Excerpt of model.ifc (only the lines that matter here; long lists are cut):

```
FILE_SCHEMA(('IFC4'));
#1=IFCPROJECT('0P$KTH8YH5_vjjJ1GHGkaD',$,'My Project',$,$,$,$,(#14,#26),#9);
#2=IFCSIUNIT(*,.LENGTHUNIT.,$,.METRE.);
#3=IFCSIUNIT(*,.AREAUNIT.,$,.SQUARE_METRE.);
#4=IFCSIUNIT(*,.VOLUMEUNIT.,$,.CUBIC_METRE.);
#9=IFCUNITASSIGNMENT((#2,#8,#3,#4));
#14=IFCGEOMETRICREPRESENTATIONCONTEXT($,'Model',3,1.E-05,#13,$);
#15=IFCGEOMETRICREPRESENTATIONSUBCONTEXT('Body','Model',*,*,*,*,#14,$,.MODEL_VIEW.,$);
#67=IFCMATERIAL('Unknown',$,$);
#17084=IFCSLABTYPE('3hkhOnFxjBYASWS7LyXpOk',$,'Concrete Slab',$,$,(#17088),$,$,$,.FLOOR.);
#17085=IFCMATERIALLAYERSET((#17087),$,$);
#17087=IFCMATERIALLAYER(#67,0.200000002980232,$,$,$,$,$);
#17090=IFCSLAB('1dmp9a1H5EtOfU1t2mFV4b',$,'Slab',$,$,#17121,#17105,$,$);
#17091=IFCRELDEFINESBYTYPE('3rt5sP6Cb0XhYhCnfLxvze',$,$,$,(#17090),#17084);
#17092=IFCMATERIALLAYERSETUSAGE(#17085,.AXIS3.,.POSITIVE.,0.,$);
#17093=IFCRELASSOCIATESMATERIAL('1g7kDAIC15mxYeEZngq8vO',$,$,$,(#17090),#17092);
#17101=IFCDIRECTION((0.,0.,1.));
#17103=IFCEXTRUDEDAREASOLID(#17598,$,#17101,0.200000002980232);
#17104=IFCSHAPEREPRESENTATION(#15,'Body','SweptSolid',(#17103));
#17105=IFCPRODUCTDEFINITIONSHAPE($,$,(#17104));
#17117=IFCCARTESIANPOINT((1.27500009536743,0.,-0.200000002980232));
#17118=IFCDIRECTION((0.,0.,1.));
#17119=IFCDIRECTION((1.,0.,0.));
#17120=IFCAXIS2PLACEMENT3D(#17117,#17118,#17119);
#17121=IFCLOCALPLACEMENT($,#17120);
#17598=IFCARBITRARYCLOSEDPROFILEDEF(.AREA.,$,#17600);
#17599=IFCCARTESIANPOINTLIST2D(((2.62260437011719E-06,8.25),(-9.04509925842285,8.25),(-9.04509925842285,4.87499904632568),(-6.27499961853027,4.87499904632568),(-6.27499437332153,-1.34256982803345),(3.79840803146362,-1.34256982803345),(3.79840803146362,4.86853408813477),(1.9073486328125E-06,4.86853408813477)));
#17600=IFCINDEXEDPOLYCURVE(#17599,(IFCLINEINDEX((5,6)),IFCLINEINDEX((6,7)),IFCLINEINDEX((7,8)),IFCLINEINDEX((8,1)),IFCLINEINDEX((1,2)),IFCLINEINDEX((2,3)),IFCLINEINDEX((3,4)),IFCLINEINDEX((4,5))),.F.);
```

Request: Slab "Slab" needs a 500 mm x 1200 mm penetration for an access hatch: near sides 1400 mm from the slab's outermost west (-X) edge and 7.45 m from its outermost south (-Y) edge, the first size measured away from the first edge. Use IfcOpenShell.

```python
import numpy as np
import ifcopenshell
import ifcopenshell.api.feature
import ifcopenshell.api.geometry
import ifcopenshell.api.root
import ifcopenshell.geom
import ifcopenshell.util.placement
import ifcopenshell.util.representation
import ifcopenshell.util.shape
import ifcopenshell.util.unit

model = ifcopenshell.open("model.ifc")
unit_scale = ifcopenshell.util.unit.calculate_unit_scale(model)
settings = ifcopenshell.geom.settings()


def volume(element):
    """Net volume in cubic metres, openings subtracted."""
    shape = ifcopenshell.geom.create_shape(settings, element)
    return ifcopenshell.util.shape.get_volume(shape.geometry)


slab = model.by_id(17090)
before = volume(slab)

# Extent in the slab's own axes, in metres. The edges named are its -X and -Y sides.
slab_shape = ifcopenshell.geom.create_shape(settings, slab)
vertices = ifcopenshell.util.shape.get_vertices(slab_shape.geometry)
x_min, y_min, bottom = vertices.min(axis=0)
top = vertices[:, 2].max()

opening = ifcopenshell.api.root.create_entity(model, ifc_class="IfcOpeningElement", name="Access hatch opening", predefined_type="OPENING")
context = ifcopenshell.util.representation.get_context(model, "Model", "Body", "MODEL_VIEW")
width, depth = 0.5, 1.2
outline = [(0.0, 0.0), (width, 0.0), (width, depth), (0.0, depth), (0.0, 0.0)]
# Overshoot both faces by 50 mm so the cut is clean.
shape = ifcopenshell.api.geometry.add_slab_representation(
    model, context=context, depth=top - bottom + 0.1, polyline=outline
)
ifcopenshell.api.geometry.assign_representation(model, product=opening, representation=shape)

matrix = ifcopenshell.util.placement.get_local_placement(slab.ObjectPlacement)
matrix[:, 3] = matrix @ np.append(np.array([x_min + 1.4, y_min + 7.45, bottom - 0.05]) / unit_scale, 1.0)
ifcopenshell.api.geometry.edit_object_placement(model, product=opening, matrix=matrix, is_si=False)
ifcopenshell.api.feature.add_feature(model, feature=opening, element=slab)

after = volume(slab)

print(f"slab volume {before:.3f} -> {after:.3f} m3")

model.write("model_updated.ifc")
```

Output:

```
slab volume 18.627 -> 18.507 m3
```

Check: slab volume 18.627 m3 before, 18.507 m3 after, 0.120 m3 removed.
